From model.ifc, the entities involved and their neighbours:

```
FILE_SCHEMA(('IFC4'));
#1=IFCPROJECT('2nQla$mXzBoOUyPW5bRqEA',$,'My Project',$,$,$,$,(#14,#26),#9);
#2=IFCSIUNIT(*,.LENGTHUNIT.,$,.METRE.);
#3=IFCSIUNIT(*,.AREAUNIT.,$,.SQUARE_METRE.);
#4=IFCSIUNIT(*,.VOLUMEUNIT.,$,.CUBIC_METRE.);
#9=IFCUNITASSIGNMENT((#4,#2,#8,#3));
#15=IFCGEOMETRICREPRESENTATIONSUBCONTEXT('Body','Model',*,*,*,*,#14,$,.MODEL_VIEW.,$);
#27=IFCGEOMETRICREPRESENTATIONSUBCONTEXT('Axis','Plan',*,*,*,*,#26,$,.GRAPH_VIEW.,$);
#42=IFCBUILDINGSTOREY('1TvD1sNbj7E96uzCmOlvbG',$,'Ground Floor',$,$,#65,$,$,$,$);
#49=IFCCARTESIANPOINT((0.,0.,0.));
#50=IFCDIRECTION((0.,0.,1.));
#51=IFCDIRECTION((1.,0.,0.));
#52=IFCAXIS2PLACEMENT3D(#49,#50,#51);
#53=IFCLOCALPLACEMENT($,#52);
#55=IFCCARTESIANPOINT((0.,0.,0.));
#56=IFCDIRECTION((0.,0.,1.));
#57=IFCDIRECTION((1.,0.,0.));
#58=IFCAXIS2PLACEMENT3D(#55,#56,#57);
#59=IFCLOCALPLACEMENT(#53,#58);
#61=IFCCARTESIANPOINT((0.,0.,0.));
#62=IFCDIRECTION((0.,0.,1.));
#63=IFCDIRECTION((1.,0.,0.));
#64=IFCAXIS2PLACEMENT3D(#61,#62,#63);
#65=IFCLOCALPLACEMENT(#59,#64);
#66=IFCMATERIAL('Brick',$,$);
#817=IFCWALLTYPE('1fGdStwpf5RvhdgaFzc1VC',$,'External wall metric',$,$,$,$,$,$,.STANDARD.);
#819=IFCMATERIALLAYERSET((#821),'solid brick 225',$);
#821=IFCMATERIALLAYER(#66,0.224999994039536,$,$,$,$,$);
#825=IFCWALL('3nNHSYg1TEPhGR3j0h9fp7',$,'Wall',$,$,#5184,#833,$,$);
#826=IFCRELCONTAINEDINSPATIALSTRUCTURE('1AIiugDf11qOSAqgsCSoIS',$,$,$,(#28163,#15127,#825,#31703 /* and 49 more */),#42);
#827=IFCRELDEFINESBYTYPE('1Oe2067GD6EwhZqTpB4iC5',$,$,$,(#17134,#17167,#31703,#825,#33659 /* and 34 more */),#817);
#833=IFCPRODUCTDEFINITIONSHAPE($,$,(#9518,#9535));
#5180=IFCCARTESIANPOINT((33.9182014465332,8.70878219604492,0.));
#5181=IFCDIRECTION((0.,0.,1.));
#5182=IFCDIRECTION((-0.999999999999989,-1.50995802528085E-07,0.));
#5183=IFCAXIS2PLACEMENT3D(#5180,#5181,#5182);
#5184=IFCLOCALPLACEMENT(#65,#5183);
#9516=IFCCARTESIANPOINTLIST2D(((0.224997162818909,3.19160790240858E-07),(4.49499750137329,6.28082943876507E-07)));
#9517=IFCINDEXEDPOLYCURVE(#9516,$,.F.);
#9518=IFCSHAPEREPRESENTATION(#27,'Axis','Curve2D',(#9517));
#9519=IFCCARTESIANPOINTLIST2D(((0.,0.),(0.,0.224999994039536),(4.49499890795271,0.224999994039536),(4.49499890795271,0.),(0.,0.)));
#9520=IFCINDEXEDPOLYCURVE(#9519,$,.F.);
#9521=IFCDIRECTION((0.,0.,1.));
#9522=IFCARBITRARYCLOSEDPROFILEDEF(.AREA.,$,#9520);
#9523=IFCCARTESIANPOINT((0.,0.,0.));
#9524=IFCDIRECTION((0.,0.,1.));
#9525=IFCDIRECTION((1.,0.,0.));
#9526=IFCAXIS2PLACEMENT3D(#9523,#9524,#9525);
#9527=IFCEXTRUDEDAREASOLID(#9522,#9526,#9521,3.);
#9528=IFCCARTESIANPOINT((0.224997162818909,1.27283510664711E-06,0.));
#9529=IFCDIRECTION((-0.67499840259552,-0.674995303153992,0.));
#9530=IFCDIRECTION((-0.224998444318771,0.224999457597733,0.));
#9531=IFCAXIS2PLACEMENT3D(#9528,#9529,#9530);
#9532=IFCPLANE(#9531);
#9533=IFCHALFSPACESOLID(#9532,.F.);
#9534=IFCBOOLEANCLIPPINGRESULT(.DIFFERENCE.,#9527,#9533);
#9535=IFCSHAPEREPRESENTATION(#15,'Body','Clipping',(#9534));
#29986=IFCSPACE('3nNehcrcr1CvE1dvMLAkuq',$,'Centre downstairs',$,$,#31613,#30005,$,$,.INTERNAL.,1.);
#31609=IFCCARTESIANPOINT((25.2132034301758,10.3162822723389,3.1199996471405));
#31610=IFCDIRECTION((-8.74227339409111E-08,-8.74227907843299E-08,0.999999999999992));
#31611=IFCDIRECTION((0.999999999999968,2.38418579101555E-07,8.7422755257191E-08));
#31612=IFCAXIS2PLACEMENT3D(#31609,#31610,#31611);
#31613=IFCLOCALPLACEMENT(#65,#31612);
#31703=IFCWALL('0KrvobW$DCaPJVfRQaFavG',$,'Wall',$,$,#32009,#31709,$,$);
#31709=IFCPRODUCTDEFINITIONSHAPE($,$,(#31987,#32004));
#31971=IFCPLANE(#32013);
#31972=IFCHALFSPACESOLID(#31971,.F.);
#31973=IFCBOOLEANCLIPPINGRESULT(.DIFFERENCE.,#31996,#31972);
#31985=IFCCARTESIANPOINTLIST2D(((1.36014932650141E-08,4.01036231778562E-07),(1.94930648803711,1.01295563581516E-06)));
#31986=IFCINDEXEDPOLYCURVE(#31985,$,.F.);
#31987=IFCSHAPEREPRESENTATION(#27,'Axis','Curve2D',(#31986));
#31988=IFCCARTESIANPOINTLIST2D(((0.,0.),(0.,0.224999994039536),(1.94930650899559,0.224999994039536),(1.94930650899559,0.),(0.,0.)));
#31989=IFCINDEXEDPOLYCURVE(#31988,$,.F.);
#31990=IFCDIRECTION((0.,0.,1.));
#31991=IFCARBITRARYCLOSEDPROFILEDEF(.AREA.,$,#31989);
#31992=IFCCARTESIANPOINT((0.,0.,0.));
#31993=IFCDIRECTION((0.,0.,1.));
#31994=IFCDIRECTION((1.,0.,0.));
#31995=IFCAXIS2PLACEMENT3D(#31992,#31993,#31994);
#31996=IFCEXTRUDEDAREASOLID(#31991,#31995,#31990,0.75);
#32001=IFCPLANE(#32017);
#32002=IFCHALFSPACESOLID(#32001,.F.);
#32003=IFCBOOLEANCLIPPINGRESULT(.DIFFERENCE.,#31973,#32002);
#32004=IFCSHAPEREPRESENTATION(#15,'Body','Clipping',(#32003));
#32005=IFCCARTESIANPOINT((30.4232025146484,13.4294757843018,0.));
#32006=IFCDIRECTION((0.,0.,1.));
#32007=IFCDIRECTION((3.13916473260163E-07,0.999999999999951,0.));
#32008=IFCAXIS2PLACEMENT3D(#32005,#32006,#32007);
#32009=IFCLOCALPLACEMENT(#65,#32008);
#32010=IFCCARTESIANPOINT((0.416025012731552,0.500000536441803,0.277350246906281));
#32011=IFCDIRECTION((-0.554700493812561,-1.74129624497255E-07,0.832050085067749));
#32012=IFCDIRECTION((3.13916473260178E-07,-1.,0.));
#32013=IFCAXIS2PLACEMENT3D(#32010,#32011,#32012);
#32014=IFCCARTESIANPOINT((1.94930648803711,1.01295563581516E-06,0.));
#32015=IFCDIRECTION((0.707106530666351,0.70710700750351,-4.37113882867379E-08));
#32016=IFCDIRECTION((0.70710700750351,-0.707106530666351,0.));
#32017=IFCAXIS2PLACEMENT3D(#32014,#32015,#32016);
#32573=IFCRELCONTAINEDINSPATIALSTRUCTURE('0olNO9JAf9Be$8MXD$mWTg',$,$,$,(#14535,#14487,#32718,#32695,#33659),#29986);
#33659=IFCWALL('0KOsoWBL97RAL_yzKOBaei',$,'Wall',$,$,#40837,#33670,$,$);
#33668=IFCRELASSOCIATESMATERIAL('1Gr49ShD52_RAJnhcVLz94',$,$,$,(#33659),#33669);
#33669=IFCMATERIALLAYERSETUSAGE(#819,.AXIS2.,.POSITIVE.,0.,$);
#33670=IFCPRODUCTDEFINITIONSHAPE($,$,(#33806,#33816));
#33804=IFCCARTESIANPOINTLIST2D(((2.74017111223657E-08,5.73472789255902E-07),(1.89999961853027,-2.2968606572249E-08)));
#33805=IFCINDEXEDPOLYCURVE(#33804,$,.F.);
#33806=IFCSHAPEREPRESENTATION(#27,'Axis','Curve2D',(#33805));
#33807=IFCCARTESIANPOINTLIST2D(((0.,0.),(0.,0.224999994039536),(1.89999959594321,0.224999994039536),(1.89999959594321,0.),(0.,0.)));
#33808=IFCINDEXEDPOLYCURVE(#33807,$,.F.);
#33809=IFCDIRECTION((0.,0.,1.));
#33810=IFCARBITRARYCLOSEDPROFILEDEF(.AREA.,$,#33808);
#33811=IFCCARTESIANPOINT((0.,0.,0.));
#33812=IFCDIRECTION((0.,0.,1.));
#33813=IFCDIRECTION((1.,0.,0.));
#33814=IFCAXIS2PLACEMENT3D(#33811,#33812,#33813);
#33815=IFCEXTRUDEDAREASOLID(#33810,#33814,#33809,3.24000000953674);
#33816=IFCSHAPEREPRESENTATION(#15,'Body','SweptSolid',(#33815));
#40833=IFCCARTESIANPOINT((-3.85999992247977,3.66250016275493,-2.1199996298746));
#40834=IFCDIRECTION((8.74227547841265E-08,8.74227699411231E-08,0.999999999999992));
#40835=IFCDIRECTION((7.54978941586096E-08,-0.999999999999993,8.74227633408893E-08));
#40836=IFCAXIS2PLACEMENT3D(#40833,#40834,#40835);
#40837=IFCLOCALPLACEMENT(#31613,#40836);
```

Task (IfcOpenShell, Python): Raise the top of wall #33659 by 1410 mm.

```python
import ifcopenshell
import ifcopenshell.geom
import ifcopenshell.util.representation
import ifcopenshell.util.shape

model = ifcopenshell.open("model.ifc")
settings = ifcopenshell.geom.settings()


def volume(element):
    """Net volume in cubic metres, openings subtracted."""
    shape = ifcopenshell.geom.create_shape(settings, element)
    return ifcopenshell.util.shape.get_volume(shape.geometry)


wall = model.by_guid("0KOsoWBL97RAL_yzKOBaei")
before = volume(wall)

body = ifcopenshell.util.representation.get_representation(wall, "Model", "Body")
solid = body.Items[0]
old_height = solid.Depth
solid.Depth += 1.41
after = volume(wall)

print(f"height {old_height:g} -> {solid.Depth:g}, volume {before:.3f} -> {after:.3f} m3")

model.write("model_rev.ifc")
```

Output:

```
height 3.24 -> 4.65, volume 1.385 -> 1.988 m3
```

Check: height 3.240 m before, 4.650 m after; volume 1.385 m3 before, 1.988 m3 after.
